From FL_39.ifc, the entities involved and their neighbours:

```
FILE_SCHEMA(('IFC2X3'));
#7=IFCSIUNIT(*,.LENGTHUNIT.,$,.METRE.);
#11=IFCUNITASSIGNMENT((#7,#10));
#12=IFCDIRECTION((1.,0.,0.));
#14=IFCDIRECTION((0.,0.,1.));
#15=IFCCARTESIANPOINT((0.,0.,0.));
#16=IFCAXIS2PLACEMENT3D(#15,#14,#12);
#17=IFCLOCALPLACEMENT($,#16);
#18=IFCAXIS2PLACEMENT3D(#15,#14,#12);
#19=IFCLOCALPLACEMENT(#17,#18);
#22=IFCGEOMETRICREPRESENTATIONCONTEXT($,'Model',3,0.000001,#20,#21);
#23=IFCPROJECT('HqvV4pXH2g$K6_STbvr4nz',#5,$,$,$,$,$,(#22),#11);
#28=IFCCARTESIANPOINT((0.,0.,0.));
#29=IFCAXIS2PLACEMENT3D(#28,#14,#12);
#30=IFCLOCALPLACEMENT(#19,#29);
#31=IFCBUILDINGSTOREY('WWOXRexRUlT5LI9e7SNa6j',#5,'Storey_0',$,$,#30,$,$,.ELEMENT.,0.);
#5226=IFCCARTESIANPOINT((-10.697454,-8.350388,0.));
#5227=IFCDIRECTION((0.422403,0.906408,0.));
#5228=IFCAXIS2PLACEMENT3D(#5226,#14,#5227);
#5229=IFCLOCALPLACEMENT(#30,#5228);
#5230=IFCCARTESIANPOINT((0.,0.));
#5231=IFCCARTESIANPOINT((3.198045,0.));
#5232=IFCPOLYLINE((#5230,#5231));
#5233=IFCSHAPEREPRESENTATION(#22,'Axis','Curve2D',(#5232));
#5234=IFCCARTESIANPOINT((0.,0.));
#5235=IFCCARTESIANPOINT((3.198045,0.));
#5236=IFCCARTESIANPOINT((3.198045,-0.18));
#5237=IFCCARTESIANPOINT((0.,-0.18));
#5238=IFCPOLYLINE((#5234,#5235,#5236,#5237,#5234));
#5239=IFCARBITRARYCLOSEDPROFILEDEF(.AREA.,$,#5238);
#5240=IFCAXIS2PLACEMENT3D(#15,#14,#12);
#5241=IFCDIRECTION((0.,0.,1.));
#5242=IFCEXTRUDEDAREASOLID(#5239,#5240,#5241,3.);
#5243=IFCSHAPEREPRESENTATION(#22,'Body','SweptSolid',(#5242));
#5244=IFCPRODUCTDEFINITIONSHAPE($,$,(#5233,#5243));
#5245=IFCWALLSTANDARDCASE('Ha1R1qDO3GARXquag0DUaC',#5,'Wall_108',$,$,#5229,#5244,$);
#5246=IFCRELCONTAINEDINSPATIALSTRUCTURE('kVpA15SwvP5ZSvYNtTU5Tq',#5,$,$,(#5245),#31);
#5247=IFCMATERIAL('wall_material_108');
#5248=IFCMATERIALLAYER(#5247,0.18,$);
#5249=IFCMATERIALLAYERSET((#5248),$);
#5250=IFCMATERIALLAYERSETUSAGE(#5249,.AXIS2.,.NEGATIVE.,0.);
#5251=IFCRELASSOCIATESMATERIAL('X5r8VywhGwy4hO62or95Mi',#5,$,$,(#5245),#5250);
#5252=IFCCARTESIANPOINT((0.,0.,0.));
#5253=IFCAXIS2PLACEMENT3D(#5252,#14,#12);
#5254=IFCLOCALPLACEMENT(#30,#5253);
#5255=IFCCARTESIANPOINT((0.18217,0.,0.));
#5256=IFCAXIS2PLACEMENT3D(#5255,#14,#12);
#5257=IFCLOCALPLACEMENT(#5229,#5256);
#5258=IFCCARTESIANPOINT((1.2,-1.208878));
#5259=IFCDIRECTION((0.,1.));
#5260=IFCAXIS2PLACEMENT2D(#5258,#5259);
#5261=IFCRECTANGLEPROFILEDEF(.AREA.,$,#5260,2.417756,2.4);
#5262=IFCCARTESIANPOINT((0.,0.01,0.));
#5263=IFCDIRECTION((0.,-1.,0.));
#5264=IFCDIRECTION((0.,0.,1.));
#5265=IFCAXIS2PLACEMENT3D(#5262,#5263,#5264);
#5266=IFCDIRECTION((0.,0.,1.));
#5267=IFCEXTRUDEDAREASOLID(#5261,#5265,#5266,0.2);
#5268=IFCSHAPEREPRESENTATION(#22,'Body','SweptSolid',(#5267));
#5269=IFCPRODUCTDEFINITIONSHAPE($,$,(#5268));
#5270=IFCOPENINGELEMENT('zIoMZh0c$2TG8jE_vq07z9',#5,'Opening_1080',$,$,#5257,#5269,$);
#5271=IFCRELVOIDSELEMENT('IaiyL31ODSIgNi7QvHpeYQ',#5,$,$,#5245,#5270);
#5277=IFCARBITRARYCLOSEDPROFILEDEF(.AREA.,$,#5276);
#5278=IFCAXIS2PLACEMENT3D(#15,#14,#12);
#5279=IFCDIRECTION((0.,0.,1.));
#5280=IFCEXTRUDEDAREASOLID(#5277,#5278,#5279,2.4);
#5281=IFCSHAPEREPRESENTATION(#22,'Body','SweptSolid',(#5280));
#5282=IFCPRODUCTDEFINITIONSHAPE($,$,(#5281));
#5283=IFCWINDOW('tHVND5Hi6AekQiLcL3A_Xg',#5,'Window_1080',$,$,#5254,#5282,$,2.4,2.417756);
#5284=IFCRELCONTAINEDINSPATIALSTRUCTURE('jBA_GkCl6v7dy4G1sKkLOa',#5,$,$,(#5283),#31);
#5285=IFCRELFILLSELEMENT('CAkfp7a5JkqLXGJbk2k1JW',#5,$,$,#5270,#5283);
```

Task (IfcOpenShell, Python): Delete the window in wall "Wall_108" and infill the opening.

```python
import ifcopenshell
import ifcopenshell.api.feature
import ifcopenshell.api.root
import ifcopenshell.geom
import ifcopenshell.util.shape

model = ifcopenshell.open("FL_39.ifc")
settings = ifcopenshell.geom.settings()


def volume(element):
    """Net volume in cubic metres, openings subtracted."""
    shape = ifcopenshell.geom.create_shape(settings, element)
    return ifcopenshell.util.shape.get_volume(shape.geometry)


window = model.by_guid("tHVND5Hi6AekQiLcL3A_Xg")
opening = window.FillsVoids[0].RelatingOpeningElement
wall = opening.VoidsElements[0].RelatingBuildingElement
before = volume(wall)

ifcopenshell.api.root.remove_product(model, product=window)
ifcopenshell.api.feature.remove_feature(model, feature=opening)

after = volume(wall)

print(f"wall volume {before:.3f} -> {after:.3f} m3")

model.write("FL_39_v2.ifc")
```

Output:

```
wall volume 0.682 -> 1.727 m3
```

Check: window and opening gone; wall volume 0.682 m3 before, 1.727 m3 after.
